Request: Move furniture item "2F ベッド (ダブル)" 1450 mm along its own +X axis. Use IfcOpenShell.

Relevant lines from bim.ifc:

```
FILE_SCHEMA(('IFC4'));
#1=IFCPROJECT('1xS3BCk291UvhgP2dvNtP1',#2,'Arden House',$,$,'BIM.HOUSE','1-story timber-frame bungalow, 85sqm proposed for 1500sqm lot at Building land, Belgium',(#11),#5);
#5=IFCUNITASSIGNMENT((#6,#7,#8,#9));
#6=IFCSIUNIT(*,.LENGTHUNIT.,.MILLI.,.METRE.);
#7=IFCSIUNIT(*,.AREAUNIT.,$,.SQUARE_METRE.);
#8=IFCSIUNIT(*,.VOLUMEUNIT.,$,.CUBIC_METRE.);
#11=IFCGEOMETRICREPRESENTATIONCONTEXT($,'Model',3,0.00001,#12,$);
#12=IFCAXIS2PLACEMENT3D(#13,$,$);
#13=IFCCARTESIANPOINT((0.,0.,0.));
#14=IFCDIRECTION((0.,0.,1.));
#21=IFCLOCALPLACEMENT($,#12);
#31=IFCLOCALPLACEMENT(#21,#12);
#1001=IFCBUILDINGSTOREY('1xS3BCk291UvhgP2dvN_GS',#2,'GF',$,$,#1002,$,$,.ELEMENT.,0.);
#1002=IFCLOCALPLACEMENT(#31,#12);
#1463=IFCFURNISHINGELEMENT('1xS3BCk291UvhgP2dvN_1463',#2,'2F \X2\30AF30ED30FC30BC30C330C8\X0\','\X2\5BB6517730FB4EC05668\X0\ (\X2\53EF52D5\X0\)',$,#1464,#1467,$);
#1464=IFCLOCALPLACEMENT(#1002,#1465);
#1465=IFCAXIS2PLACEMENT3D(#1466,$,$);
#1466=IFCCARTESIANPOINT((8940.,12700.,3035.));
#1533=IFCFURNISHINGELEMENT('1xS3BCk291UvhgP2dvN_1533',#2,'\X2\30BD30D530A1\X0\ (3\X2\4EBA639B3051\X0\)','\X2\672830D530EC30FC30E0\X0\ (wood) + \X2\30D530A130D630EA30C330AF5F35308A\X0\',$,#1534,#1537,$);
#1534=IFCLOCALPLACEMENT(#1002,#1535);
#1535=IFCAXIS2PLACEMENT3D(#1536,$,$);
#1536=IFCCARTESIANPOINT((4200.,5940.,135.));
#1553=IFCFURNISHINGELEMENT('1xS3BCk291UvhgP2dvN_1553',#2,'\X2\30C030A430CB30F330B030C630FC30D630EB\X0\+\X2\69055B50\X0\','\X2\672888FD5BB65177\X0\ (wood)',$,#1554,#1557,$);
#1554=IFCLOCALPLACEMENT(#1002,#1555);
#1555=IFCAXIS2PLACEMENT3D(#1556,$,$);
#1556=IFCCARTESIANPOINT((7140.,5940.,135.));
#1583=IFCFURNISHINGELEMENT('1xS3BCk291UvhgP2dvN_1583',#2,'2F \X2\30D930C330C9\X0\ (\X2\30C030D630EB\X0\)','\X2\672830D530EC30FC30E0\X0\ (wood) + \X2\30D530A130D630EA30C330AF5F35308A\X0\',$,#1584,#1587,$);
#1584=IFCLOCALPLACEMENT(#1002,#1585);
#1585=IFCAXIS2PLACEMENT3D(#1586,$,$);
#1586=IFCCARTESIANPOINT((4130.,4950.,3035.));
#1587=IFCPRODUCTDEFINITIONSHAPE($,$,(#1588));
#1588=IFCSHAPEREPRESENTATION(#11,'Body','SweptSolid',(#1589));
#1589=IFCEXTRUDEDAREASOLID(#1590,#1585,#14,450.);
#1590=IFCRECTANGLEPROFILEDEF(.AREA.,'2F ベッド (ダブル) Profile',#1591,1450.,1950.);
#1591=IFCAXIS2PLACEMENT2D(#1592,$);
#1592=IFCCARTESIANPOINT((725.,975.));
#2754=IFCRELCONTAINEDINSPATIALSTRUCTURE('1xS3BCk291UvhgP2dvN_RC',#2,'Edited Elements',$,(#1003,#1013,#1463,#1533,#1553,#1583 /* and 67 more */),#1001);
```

```python
import ifcopenshell
import ifcopenshell.api.geometry
import ifcopenshell.util.placement
import ifcopenshell.util.unit

model = ifcopenshell.open("bim.ifc")
unit_scale = ifcopenshell.util.unit.calculate_unit_scale(model)

item = model.by_guid("1xS3BCk291UvhgP2dvN_1583")
matrix = ifcopenshell.util.placement.get_local_placement(item.ObjectPlacement)
matrix[:3, 3] += matrix[:3, 0] * 1.45 / unit_scale
ifcopenshell.api.geometry.edit_object_placement(model, product=item, matrix=matrix, is_si=False)

print(ifcopenshell.util.placement.get_local_placement(item.ObjectPlacement).round(3) + 0.0)

model.write("bim_edited.ifc")
```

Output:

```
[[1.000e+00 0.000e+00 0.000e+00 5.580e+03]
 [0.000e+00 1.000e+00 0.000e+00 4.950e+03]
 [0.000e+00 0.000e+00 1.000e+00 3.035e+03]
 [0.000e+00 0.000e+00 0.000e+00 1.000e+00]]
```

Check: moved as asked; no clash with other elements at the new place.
